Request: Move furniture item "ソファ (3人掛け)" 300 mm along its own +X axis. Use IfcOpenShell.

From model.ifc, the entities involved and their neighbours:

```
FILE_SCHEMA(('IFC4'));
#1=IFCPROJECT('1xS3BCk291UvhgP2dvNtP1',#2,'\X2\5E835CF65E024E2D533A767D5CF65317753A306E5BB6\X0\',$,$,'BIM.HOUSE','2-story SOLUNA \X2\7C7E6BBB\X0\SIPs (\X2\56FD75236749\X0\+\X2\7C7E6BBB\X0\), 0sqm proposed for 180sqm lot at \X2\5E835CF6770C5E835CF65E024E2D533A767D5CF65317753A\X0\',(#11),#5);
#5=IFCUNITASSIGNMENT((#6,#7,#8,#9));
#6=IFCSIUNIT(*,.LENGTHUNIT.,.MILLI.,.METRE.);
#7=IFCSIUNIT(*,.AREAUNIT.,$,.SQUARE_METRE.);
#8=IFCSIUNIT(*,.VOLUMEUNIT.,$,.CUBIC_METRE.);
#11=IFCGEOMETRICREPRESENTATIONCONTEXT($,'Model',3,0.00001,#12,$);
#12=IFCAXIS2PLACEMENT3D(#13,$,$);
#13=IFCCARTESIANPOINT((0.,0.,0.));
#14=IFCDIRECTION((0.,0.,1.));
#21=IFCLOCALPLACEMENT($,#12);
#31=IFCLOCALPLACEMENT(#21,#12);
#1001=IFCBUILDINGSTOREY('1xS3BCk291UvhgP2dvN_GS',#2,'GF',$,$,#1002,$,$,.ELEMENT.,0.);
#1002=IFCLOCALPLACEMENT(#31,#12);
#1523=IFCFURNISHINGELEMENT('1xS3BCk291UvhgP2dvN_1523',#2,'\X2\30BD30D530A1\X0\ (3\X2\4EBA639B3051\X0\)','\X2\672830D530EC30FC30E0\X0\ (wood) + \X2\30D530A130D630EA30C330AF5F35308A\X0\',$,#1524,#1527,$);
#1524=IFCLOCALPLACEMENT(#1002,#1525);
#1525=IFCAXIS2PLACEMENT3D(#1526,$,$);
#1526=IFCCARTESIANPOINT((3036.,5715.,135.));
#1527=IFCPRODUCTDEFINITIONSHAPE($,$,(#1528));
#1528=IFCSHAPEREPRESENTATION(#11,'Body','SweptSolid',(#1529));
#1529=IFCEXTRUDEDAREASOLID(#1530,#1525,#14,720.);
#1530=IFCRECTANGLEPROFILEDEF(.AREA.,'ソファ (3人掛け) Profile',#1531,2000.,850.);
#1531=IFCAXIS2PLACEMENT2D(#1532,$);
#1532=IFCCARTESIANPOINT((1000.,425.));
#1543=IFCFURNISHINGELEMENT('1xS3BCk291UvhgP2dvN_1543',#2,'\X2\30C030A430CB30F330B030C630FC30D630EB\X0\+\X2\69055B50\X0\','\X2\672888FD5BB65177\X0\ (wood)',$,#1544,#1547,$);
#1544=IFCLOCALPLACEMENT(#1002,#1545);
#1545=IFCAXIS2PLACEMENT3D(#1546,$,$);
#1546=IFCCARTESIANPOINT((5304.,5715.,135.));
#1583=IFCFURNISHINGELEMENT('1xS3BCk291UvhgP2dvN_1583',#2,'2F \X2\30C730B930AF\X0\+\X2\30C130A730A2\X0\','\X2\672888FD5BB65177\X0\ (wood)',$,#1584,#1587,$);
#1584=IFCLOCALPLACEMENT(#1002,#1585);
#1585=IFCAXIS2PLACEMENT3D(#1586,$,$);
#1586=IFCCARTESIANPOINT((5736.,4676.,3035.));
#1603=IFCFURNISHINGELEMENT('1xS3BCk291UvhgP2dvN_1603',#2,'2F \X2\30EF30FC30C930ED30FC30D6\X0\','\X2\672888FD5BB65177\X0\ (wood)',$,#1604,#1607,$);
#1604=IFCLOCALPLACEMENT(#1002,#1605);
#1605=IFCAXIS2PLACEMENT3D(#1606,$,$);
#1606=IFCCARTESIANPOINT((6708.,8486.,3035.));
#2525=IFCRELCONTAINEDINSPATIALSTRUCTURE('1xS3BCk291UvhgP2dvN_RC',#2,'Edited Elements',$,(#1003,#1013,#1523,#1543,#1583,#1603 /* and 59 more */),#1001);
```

```python
import ifcopenshell
import ifcopenshell.api.geometry
import ifcopenshell.util.placement

model = ifcopenshell.open("model.ifc")

item = model.by_id(1523)
matrix = ifcopenshell.util.placement.get_local_placement(item.ObjectPlacement)
matrix[:3, 3] += matrix[:3, 0] * 300.0
ifcopenshell.api.geometry.edit_object_placement(model, product=item, matrix=matrix, is_si=False)

print(ifcopenshell.util.placement.get_local_placement(item.ObjectPlacement).round(3) + 0.0)

model.write("model_updated.ifc")
```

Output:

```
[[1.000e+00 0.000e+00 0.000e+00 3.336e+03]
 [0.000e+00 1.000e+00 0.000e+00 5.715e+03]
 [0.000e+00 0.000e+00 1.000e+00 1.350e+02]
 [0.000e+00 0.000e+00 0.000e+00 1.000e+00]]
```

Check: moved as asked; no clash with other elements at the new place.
